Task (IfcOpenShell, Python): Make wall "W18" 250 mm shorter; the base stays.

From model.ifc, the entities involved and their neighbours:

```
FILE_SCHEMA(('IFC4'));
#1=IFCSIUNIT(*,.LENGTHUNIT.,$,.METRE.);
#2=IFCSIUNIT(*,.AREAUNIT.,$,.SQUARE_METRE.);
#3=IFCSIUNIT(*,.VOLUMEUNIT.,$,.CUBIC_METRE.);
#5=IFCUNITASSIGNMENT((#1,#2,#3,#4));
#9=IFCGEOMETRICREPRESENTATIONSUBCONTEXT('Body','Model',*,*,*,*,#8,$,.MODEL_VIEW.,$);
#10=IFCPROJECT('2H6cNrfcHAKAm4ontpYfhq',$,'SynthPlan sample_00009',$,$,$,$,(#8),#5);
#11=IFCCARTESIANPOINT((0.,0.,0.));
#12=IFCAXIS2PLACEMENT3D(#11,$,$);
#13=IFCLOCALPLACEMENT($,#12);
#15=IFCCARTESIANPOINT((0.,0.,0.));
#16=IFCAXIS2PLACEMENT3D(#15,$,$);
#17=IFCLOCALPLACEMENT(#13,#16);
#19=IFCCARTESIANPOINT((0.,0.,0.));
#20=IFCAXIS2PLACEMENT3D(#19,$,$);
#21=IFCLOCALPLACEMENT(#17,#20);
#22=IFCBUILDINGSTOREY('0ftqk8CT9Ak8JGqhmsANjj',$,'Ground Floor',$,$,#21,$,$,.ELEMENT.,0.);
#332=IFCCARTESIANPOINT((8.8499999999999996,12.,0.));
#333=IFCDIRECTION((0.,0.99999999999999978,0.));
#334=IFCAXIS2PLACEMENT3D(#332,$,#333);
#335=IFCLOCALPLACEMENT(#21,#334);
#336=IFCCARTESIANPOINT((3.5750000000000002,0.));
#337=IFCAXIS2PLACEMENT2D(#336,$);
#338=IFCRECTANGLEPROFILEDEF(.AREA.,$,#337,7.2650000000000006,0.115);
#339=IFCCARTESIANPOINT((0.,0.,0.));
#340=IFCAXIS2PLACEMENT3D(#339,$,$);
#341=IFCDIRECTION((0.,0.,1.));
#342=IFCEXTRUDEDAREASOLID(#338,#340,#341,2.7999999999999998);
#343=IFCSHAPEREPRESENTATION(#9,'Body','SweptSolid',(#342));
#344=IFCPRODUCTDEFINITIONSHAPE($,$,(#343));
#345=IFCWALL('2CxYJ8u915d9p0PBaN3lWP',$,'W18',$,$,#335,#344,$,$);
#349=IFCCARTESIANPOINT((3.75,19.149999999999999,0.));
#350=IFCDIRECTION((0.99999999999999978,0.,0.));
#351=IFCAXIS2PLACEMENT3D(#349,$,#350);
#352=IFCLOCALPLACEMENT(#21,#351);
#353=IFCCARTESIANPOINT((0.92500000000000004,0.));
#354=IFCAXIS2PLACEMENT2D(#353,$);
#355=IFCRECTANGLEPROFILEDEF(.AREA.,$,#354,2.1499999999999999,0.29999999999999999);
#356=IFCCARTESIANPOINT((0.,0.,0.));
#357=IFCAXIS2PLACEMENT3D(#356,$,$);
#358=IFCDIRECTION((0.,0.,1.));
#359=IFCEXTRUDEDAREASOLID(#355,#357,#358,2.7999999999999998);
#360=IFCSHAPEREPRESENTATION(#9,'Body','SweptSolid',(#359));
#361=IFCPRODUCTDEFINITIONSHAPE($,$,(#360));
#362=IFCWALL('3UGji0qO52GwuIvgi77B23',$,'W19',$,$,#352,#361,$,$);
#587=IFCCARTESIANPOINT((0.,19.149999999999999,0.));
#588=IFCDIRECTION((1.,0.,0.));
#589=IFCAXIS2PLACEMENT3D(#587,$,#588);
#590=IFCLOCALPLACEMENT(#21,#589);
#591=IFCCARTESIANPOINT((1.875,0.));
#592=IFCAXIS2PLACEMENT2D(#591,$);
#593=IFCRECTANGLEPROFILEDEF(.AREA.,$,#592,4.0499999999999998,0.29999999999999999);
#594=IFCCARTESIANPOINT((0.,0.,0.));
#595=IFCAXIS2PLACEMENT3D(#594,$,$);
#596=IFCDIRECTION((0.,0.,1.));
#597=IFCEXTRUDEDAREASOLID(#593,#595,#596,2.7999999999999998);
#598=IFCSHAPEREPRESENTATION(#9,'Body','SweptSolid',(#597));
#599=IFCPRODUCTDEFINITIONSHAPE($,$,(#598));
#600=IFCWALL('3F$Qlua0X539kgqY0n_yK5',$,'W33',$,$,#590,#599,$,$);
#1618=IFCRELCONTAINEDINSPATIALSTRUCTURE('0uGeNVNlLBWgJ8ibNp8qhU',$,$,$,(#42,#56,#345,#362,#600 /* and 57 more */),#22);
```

```python
import ifcopenshell
import ifcopenshell.geom
import ifcopenshell.util.representation
import ifcopenshell.util.shape
import ifcopenshell.util.unit

model = ifcopenshell.open("model.ifc")
unit_scale = ifcopenshell.util.unit.calculate_unit_scale(model)
settings = ifcopenshell.geom.settings()


def volume(element):
    """Net volume in cubic metres, openings subtracted."""
    shape = ifcopenshell.geom.create_shape(settings, element)
    return ifcopenshell.util.shape.get_volume(shape.geometry)


wall = model.by_id(345)
before = volume(wall)

body = ifcopenshell.util.representation.get_representation(wall, "Model", "Body")
solid = body.Items[0]
old_height = solid.Depth
solid.Depth -= 0.25 / unit_scale
after = volume(wall)

print(f"height {old_height:g} -> {solid.Depth:g}, volume {before:.3f} -> {after:.3f} m3")

model.write("model_updated.ifc")
```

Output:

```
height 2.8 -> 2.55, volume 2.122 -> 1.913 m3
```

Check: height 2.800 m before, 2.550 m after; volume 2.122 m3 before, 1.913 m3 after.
